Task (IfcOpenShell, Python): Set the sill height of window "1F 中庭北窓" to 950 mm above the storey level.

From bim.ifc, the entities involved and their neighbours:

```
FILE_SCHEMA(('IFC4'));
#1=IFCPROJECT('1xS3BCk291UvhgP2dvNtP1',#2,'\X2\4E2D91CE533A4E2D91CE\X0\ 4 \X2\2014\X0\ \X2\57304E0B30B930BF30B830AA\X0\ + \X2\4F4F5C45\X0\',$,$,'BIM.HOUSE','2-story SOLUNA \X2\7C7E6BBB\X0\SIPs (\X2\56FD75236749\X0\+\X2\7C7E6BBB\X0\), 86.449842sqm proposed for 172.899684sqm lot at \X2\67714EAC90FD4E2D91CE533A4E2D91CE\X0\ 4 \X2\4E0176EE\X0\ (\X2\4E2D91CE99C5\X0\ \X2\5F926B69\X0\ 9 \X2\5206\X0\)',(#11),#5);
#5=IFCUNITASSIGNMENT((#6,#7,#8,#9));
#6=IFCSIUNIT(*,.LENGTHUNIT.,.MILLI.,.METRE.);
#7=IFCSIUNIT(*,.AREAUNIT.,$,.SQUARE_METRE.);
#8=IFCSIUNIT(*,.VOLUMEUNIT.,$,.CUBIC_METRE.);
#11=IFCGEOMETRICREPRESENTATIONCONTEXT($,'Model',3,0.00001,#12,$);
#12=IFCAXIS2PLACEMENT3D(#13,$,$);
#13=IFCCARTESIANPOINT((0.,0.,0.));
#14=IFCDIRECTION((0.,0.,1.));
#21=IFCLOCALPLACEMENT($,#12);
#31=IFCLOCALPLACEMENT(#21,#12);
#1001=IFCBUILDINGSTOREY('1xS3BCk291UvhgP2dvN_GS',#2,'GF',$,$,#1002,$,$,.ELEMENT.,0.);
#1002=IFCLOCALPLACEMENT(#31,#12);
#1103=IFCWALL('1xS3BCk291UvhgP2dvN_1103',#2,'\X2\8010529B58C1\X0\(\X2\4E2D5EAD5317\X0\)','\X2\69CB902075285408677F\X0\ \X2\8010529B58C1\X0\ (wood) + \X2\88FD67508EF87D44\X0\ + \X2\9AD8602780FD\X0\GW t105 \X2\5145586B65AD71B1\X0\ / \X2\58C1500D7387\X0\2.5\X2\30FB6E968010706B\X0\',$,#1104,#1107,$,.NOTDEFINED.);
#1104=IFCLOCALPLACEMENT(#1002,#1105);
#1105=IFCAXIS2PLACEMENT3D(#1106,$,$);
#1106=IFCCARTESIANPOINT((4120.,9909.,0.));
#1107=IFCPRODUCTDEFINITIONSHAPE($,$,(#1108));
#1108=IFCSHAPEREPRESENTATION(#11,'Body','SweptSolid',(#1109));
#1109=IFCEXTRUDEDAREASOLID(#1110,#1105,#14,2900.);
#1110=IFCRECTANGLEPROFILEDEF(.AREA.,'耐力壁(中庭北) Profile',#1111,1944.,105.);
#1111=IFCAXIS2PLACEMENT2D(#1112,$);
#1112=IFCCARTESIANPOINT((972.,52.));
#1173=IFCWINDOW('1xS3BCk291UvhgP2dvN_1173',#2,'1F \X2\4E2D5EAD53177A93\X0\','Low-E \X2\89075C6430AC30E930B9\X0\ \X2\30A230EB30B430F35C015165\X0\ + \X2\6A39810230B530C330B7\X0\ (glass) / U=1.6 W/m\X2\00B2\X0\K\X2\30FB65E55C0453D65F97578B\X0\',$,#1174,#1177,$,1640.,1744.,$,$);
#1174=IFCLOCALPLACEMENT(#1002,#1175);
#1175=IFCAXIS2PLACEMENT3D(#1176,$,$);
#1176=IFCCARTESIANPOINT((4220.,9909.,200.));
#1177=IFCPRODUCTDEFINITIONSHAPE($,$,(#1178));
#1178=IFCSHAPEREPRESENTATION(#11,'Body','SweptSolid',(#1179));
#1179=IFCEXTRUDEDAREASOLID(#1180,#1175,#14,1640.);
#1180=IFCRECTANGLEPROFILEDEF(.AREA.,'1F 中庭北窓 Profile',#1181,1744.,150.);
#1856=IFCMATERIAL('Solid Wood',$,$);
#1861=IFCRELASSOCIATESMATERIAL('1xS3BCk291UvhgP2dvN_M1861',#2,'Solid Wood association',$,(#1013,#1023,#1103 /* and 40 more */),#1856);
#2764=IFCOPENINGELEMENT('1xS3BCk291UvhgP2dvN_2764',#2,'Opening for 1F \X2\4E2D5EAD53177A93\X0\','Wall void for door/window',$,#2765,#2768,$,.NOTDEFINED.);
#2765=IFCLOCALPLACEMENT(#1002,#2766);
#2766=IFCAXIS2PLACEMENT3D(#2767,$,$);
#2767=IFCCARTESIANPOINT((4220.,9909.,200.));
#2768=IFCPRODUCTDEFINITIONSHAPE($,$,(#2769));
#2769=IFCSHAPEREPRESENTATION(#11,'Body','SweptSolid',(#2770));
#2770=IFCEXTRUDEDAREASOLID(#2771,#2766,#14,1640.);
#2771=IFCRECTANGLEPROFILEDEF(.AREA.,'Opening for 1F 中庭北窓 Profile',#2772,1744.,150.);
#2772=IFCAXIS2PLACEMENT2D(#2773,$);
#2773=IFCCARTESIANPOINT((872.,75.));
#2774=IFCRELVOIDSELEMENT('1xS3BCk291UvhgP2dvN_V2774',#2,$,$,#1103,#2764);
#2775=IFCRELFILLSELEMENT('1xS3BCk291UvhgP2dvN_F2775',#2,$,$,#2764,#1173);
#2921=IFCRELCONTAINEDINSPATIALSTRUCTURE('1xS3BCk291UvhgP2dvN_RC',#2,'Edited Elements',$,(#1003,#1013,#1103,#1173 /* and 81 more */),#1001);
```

```python
import numpy as np
import ifcopenshell
import ifcopenshell.api.geometry
import ifcopenshell.geom
import ifcopenshell.util.element
import ifcopenshell.util.placement
import ifcopenshell.util.shape
import ifcopenshell.util.unit

model = ifcopenshell.open("bim.ifc")
unit_scale = ifcopenshell.util.unit.calculate_unit_scale(model)

window = model.by_guid("1xS3BCk291UvhgP2dvN_1173")
opening = window.FillsVoids[0].RelatingOpeningElement
storey = ifcopenshell.util.element.get_container(window, ifc_class="IfcBuildingStorey")
level = ifcopenshell.util.placement.get_local_placement(storey.ObjectPlacement)[2, 3]

# The opening's origin need not be at the sill, so measure its lowest point.
shape = ifcopenshell.geom.create_shape(ifcopenshell.geom.settings(), opening)
bottom = ifcopenshell.util.shape.get_shape_bottom_elevation(shape, shape.geometry) / unit_scale
dz = level + 0.95 / unit_scale - bottom

shift = np.array([0.0, 0.0, dz])
# The window is not placed relative to its opening, so move both.
for product in (opening, window):
    matrix = ifcopenshell.util.placement.get_local_placement(product.ObjectPlacement)
    matrix[:3, 3] += shift
    ifcopenshell.api.geometry.edit_object_placement(model, product=product, matrix=matrix, is_si=False)

print(f"moved by {dz * unit_scale:+.3f} m")

model.write("bim_updated.ifc")
```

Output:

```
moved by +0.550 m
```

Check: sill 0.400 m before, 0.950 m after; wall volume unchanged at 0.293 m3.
